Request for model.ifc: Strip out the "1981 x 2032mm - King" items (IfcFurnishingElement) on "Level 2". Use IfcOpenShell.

First a look at what the model holds.

```python
import ifcopenshell
import ifcopenshell.util.element

model = ifcopenshell.open("model.ifc")
print(model.schema)
storey = next(s for s in model.by_type("IfcBuildingStorey") if s.Name == "Level 2")
furniture = [e for e in ifcopenshell.util.element.get_decomposition(storey) if e.is_a("IfcFurnishingElement")]
seen = {}
for e in furniture:
    element_type = ifcopenshell.util.element.get_type(e)
    name = element_type.Name if element_type not in (None, e) else None
    seen[name] = seen.get(name, 0) + 1
for name, count in sorted(seen.items(), key=str):
    print(count, "x", name)
```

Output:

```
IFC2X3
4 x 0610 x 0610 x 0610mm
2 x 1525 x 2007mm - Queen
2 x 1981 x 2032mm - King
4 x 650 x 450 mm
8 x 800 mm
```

```python
import ifcopenshell
import ifcopenshell.api.root
import ifcopenshell.util.element

model = ifcopenshell.open("model.ifc")

storey = next(s for s in model.by_type("IfcBuildingStorey") if s.Name == "Level 2")
furniture = [e for e in ifcopenshell.util.element.get_decomposition(storey) if e.is_a("IfcFurnishingElement")]
targets = [e for e in furniture if (t := ifcopenshell.util.element.get_type(e)) not in (None, e) and t.Name == "1981 x 2032mm - King"]

for e in targets:
    ifcopenshell.api.root.remove_product(model, product=e)
print(len(targets), "removed")

model.write("model-out.ifc")
```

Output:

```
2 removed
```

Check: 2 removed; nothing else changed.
